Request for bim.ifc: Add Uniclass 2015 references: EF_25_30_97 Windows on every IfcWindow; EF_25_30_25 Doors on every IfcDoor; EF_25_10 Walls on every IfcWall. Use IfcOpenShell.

First a look at what the model holds.

```python
import ifcopenshell

model = ifcopenshell.open("bim.ifc")
print(model.schema)
print("classifications:", [c.Name for c in model.by_type("IfcClassification")])
for ifc_class in ("IfcDoor", "IfcRoof", "IfcStair", "IfcWall", "IfcWindow"):
    print(ifc_class, len(model.by_type(ifc_class)))
```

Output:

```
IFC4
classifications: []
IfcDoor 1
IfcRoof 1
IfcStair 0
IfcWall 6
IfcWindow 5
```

```python
import ifcopenshell
import ifcopenshell.api.classification

model = ifcopenshell.open("bim.ifc")

system = ifcopenshell.api.classification.add_classification(model, classification="Uniclass 2015")

codes = {
    "IfcWindow": ("EF_25_30_97", "Windows"),
    "IfcDoor": ("EF_25_30_25", "Doors"),
    "IfcWall": ("EF_25_10", "Walls"),
}
for ifc_class, (code, name) in codes.items():
    products = model.by_type(ifc_class)
    ifcopenshell.api.classification.add_reference(
        model, products=products, classification=system, identification=code, name=name
    )
    print(code, len(products))

model.write("bim_v2.ifc")
```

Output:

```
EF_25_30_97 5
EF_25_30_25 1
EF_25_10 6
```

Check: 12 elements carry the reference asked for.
